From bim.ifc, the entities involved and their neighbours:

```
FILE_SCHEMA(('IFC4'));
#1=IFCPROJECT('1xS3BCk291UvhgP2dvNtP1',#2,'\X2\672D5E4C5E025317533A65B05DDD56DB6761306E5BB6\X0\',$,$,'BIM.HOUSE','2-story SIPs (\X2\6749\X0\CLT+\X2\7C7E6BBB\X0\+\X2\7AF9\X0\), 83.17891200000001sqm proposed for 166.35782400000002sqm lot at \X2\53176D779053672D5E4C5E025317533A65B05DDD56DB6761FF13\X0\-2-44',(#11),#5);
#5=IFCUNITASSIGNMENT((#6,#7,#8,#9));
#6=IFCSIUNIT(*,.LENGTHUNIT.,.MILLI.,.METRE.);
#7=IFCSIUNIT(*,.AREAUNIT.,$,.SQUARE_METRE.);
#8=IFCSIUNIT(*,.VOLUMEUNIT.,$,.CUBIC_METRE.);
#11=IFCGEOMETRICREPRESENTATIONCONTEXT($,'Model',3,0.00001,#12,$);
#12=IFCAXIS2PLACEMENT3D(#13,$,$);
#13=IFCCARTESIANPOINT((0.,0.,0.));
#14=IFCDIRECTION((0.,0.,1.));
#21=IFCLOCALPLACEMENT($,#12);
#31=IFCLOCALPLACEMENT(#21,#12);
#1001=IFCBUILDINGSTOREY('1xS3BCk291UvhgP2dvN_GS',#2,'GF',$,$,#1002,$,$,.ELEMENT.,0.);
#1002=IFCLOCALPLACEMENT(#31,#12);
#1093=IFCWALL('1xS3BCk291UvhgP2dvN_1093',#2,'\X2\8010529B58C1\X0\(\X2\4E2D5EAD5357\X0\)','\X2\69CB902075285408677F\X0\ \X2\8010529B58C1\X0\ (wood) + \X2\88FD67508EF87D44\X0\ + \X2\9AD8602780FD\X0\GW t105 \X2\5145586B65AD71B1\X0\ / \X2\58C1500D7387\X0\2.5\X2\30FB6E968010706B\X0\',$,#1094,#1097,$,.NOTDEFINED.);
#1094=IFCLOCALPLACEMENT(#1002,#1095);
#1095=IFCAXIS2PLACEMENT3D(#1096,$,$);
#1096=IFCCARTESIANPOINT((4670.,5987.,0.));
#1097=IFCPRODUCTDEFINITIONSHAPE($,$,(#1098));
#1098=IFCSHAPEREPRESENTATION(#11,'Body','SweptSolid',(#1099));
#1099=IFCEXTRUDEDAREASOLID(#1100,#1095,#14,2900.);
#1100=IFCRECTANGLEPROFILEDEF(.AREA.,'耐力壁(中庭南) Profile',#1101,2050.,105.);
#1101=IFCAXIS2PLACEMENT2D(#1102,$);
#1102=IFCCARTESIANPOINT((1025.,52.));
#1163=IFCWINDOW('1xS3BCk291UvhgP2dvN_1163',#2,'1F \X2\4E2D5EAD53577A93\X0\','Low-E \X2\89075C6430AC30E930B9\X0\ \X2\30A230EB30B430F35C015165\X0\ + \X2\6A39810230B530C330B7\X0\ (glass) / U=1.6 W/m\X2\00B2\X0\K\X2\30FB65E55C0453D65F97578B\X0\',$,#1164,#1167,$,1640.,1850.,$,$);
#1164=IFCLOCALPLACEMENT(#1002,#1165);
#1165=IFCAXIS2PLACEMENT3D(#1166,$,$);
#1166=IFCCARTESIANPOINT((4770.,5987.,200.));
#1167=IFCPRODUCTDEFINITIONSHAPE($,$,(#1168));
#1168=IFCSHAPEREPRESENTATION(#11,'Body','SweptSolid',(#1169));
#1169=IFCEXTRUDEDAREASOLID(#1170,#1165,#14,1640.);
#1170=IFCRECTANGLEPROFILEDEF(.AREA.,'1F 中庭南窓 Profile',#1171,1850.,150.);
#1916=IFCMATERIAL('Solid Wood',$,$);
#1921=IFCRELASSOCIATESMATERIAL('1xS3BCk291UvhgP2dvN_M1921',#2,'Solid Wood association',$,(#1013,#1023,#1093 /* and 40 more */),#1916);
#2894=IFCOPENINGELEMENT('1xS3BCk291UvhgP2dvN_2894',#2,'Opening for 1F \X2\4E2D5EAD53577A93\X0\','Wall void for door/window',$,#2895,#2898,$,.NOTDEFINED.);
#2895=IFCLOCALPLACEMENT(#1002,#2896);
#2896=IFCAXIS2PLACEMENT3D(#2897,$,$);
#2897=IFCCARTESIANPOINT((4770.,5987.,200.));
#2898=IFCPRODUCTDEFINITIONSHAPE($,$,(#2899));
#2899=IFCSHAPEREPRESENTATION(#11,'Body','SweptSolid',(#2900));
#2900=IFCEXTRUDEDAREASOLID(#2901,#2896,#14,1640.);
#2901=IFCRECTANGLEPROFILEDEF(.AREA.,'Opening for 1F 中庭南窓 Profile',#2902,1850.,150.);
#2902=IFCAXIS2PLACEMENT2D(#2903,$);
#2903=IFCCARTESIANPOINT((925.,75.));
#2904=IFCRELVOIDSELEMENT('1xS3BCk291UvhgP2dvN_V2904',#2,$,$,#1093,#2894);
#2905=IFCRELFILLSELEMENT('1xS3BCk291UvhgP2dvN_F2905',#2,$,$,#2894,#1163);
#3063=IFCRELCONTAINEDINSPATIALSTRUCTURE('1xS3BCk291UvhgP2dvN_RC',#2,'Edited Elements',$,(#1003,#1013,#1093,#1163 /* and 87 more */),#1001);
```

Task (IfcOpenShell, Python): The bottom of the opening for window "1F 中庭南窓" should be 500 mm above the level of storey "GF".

```python
import numpy as np
import ifcopenshell
import ifcopenshell.api.geometry
import ifcopenshell.geom
import ifcopenshell.util.element
import ifcopenshell.util.placement
import ifcopenshell.util.shape
import ifcopenshell.util.unit

model = ifcopenshell.open("bim.ifc")
unit_scale = ifcopenshell.util.unit.calculate_unit_scale(model)

window = model.by_guid("1xS3BCk291UvhgP2dvN_1163")
opening = window.FillsVoids[0].RelatingOpeningElement
storey = ifcopenshell.util.element.get_container(window, ifc_class="IfcBuildingStorey")
level = ifcopenshell.util.placement.get_local_placement(storey.ObjectPlacement)[2, 3]

# The opening's origin need not be at the sill, so measure its lowest point.
shape = ifcopenshell.geom.create_shape(ifcopenshell.geom.settings(), opening)
bottom = ifcopenshell.util.shape.get_shape_bottom_elevation(shape, shape.geometry) / unit_scale
dz = level + 500.0 - bottom

shift = np.array([0.0, 0.0, dz])
# The window is not placed relative to its opening, so move both.
for product in (opening, window):
    matrix = ifcopenshell.util.placement.get_local_placement(product.ObjectPlacement)
    matrix[:3, 3] += shift
    ifcopenshell.api.geometry.edit_object_placement(model, product=product, matrix=matrix, is_si=False)

print(f"moved by {dz * unit_scale:+.3f} m")

model.write("bim_v2.ifc")
```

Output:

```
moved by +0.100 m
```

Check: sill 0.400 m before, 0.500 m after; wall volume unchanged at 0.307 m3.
